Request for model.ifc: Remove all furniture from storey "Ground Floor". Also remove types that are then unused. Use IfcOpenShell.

First a look at what the model holds.

```python
import ifcopenshell
import ifcopenshell.util.element

model = ifcopenshell.open("model.ifc")
print(model.schema)
storey = next(s for s in model.by_type("IfcBuildingStorey") if s.Name == "Ground Floor")
furniture = [e for e in ifcopenshell.util.element.get_decomposition(storey) if e.is_a("IfcFurnishingElement")]
seen = {}
for e in furniture:
    element_type = ifcopenshell.util.element.get_type(e)
    name = element_type.Name if element_type not in (None, e) else None
    seen[name] = seen.get(name, 0) + 1
for name, count in sorted(seen.items(), key=str):
    print(count, "x", name)
```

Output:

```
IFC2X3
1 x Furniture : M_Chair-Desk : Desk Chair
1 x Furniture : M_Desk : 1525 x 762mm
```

```python
import ifcopenshell
import ifcopenshell.api.root
import ifcopenshell.util.element

model = ifcopenshell.open("model.ifc")

storey = next(s for s in model.by_type("IfcBuildingStorey") if s.Name == "Ground Floor")
furniture = [e for e in ifcopenshell.util.element.get_decomposition(storey) if e.is_a("IfcFurnishingElement")]
types = {ifcopenshell.util.element.get_type(e) for e in furniture} - {None, *furniture}

for e in furniture:
    ifcopenshell.api.root.remove_product(model, product=e)
print(len(furniture), "removed")

unused = [t for t in types if not ifcopenshell.util.element.get_types(t)]
for t in unused:
    ifcopenshell.api.root.remove_product(model, product=t)
print(len(unused), "unused types removed")

model.write("model_v2.ifc")
```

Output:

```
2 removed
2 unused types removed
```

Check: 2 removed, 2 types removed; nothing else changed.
